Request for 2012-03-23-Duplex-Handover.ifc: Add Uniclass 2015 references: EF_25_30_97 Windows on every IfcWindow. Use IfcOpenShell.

First a look at what the model holds.

```python
import ifcopenshell

model = ifcopenshell.open("2012-03-23-Duplex-Handover.ifc")
print(model.schema)
print("classifications:", [c.Name for c in model.by_type("IfcClassification")])
for ifc_class in ("IfcDoor", "IfcRoof", "IfcStair", "IfcWall", "IfcWindow"):
    print(ifc_class, len(model.by_type(ifc_class)))
```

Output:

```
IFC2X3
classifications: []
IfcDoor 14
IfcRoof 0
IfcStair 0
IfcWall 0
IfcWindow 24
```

```python
import ifcopenshell
import ifcopenshell.api.classification

model = ifcopenshell.open("2012-03-23-Duplex-Handover.ifc")

# IFC2X3 requires Source and Edition and has no link from the project to the system.
system = model.create_entity("IfcClassification", Source="NBS", Edition="2015", Name="Uniclass 2015")

codes = {
    "IfcWindow": ("EF_25_30_97", "Windows"),
}
for ifc_class, (code, name) in codes.items():
    products = model.by_type(ifc_class)
    ifcopenshell.api.classification.add_reference(
        model, products=products, classification=system, identification=code, name=name
    )
    print(code, len(products))

model.write("2012-03-23-Duplex-Handover_edited.ifc")
```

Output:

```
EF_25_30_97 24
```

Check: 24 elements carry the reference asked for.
